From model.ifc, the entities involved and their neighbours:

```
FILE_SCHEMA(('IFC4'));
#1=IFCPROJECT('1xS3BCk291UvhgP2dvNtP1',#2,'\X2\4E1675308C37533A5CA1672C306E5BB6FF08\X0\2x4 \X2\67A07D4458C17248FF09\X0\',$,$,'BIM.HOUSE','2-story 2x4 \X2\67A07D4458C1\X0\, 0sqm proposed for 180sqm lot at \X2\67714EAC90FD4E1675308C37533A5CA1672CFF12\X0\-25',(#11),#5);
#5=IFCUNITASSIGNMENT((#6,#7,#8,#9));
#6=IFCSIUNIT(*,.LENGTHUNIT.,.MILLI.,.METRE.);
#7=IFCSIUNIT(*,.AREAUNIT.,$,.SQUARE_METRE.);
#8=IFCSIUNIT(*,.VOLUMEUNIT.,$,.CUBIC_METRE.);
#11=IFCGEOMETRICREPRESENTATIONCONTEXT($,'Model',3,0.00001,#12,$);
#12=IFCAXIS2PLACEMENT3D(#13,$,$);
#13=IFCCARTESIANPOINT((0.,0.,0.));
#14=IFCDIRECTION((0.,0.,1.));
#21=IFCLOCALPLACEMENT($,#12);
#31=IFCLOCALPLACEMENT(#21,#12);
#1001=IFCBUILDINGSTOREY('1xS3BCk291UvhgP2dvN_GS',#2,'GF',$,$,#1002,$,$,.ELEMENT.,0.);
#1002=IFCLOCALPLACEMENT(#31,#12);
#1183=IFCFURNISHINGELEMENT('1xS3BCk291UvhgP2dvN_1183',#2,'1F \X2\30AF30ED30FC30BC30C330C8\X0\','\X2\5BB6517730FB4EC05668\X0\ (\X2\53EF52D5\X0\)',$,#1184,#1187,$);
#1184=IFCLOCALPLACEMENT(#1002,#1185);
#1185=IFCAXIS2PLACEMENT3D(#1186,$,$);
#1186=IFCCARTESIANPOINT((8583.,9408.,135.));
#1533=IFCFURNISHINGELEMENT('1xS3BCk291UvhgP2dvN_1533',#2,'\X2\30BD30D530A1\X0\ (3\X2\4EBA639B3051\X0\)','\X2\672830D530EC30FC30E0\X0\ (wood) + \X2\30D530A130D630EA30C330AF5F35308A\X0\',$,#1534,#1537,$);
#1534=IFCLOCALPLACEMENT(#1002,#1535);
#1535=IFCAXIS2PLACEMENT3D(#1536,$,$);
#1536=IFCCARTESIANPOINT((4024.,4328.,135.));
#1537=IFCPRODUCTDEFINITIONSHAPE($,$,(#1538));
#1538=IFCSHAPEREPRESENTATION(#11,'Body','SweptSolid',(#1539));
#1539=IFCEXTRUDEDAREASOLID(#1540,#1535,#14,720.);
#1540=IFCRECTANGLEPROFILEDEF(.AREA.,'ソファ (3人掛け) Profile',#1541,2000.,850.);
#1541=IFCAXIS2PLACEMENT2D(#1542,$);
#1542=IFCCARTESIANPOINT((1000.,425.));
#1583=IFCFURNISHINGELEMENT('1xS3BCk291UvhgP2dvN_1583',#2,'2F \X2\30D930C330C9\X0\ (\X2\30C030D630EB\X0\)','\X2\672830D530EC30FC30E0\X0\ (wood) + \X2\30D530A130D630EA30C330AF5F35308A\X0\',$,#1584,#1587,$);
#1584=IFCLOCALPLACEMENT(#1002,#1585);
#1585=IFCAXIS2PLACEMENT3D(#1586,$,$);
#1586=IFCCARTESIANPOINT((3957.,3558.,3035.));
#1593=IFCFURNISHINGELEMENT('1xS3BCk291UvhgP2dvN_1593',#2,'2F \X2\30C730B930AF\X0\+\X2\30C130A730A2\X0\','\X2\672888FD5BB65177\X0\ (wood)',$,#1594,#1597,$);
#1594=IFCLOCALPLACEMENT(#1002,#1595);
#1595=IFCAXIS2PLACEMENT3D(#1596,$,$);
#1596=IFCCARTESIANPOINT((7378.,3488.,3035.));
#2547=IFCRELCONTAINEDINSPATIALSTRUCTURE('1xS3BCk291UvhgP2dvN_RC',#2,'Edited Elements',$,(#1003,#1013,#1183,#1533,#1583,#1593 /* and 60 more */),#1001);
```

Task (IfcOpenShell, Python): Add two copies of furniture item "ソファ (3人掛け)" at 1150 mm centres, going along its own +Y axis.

```python
import ifcopenshell
import ifcopenshell.api.geometry
import ifcopenshell.api.root
import ifcopenshell.util.element
import ifcopenshell.util.placement
import ifcopenshell.util.unit

model = ifcopenshell.open("model.ifc")
unit_scale = ifcopenshell.util.unit.calculate_unit_scale(model)


def reuse_history(source, copy):
    """copy_class also copies each property set's owner history, people and application; keep the originals."""
    for rel in copy.IsDefinedBy:
        if rel.is_a("IfcRelDefinesByProperties") and (history := rel.RelatingPropertyDefinition.OwnerHistory):
            rel.RelatingPropertyDefinition.OwnerHistory = source.OwnerHistory
            ifcopenshell.util.element.remove_deep2(model, history)


source = model.by_guid("1xS3BCk291UvhgP2dvN_1533")
base = ifcopenshell.util.placement.get_local_placement(source.ObjectPlacement)
step = base[:3, 1] * 1.15 / unit_scale

for i in range(1, 3):
    copy = ifcopenshell.api.root.copy_class(model, product=source)
    copy.Representation = ifcopenshell.util.element.copy_deep(
        model, source.Representation, exclude=["IfcGeometricRepresentationContext", "IfcRepresentationMap"]
    )
    reuse_history(source, copy)
    matrix = base.copy()
    matrix[:3, 3] += i * step
    print("added at", matrix[:3, 3].round(3) + 0.0)
    ifcopenshell.api.geometry.edit_object_placement(model, product=copy, matrix=matrix, is_si=False)

model.write("model_edited.ifc")
```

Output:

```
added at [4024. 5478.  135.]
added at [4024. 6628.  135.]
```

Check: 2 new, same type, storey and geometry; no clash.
